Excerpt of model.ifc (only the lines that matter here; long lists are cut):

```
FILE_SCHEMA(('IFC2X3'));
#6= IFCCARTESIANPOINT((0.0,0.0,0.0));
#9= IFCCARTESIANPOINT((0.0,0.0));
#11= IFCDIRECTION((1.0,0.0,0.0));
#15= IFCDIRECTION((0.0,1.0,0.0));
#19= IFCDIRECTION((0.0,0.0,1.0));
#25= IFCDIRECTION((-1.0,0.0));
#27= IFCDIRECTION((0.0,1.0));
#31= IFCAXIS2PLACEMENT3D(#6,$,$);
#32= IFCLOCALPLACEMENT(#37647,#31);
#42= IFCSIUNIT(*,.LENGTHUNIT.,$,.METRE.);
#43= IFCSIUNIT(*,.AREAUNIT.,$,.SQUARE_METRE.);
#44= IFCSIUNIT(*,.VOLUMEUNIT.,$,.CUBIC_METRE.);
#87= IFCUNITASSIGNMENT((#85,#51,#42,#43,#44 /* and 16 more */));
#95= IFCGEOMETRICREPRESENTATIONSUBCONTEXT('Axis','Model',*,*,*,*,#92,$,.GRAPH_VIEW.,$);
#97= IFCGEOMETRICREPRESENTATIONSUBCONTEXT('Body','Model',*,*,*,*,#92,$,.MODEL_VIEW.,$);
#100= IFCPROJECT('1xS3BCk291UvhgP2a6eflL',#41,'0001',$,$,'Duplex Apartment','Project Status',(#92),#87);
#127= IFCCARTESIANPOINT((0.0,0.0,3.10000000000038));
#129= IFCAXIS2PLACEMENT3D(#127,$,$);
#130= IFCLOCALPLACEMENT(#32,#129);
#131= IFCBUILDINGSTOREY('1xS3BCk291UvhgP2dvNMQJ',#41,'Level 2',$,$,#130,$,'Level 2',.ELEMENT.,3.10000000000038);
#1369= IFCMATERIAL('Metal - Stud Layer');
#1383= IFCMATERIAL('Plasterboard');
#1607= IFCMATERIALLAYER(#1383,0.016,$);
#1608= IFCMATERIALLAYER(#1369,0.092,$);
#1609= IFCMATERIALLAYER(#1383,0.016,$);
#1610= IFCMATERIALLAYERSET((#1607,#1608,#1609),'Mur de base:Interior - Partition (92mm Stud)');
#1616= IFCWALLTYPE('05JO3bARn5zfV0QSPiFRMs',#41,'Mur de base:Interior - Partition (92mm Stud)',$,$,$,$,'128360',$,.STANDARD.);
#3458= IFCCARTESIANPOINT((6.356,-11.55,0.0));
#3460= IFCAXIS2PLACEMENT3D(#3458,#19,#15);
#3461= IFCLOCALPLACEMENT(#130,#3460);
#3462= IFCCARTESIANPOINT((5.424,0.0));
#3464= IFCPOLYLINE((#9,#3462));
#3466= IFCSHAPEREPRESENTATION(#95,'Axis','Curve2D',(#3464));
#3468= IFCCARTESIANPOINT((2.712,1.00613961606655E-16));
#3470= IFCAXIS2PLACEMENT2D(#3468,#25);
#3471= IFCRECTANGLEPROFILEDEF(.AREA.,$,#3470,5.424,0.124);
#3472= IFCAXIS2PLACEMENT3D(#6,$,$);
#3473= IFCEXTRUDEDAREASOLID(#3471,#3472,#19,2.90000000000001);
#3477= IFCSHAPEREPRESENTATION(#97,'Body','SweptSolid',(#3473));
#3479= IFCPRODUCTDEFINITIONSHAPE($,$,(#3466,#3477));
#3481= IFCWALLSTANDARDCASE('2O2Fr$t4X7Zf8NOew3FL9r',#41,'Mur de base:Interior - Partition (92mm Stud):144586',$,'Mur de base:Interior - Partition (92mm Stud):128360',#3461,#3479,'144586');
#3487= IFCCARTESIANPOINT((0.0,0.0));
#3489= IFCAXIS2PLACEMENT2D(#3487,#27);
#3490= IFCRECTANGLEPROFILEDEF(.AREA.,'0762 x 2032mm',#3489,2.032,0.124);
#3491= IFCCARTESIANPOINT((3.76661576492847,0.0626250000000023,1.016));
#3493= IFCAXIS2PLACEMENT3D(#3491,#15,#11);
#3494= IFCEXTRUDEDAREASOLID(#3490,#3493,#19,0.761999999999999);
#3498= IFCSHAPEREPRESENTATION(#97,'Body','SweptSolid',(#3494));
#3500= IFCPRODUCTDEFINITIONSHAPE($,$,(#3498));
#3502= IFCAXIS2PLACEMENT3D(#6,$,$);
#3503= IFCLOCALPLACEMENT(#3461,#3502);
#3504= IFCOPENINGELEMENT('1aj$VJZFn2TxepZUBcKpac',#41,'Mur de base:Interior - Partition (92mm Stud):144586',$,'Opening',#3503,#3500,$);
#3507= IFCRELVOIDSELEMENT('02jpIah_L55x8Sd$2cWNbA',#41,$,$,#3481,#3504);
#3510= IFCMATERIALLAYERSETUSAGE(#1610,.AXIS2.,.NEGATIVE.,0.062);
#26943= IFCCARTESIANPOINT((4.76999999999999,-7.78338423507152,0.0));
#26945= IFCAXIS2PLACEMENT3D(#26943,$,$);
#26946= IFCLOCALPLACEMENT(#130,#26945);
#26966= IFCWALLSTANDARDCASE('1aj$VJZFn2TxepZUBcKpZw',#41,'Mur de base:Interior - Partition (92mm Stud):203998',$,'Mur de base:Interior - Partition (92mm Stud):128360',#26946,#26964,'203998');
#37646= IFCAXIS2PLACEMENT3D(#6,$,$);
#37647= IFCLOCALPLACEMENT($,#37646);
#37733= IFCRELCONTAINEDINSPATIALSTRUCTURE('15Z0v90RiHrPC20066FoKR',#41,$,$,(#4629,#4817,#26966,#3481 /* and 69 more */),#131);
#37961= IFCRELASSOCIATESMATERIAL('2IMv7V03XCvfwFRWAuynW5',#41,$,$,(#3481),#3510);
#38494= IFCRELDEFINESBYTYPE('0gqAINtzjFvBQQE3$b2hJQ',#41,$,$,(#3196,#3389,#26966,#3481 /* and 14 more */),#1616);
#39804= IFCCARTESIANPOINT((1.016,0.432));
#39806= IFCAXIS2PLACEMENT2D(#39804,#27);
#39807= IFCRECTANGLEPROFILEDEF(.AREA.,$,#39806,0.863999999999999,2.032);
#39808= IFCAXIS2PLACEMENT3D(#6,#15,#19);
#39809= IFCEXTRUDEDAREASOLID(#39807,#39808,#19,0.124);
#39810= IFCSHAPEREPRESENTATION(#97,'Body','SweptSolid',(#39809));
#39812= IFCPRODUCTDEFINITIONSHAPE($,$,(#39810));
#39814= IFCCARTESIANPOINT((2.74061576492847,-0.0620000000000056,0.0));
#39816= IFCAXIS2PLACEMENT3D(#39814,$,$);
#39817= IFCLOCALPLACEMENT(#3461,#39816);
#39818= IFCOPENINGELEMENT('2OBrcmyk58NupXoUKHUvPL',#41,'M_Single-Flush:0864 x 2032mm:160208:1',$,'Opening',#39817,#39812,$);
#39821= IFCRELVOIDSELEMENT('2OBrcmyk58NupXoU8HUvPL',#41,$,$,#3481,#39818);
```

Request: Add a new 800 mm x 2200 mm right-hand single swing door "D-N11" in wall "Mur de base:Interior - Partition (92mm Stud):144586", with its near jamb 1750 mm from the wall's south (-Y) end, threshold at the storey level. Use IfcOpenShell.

```python
import numpy as np
import ifcopenshell
import ifcopenshell.api.feature
import ifcopenshell.api.geometry
import ifcopenshell.api.root
import ifcopenshell.api.spatial
import ifcopenshell.api.type
import ifcopenshell.geom
import ifcopenshell.util.element
import ifcopenshell.util.placement
import ifcopenshell.util.representation
import ifcopenshell.util.shape
import ifcopenshell.util.unit

model = ifcopenshell.open("model.ifc")
unit_scale = ifcopenshell.util.unit.calculate_unit_scale(model)
settings = ifcopenshell.geom.settings()


def volume(element):
    """Net volume in cubic metres, openings subtracted."""
    shape = ifcopenshell.geom.create_shape(settings, element)
    return ifcopenshell.util.shape.get_volume(shape.geometry)


wall = model.by_guid("2O2Fr$t4X7Zf8NOew3FL9r")
storey = ifcopenshell.util.element.get_container(wall, ifc_class="IfcBuildingStorey")
context = ifcopenshell.util.representation.get_context(model, "Model", "Body", "MODEL_VIEW")
before = volume(wall)

width, height, from_end, sill = 0.8, 2.2, 1.75, 0.0  # metres

# The wall runs along its own X axis, and the end named is its -X end.
wall_shape = ifcopenshell.geom.create_shape(settings, wall)
x, y, z = ifcopenshell.util.shape.get_vertices(wall_shape.geometry).T
start = x.min() + from_end
face, thickness = float(y.min()), float(y.max() - y.min())
wall_matrix = ifcopenshell.util.placement.get_local_placement(wall.ObjectPlacement)
level = ifcopenshell.util.placement.get_local_placement(storey.ObjectPlacement)[2, 3]


def in_wall(x, y):
    """Placement at x, y metres in the wall's axes, at sill height."""
    matrix = wall_matrix.copy()
    matrix[:, 3] = wall_matrix @ np.array([x / unit_scale, y / unit_scale, 0.0, 1.0])
    matrix[2, 3] = level + sill / unit_scale
    return matrix


# Opening: a box that overshoots both wall faces by 50 mm.
opening = ifcopenshell.api.root.create_entity(model, ifc_class="IfcOpeningElement")
box = ifcopenshell.api.geometry.add_wall_representation(
    model, context=context, length=width, height=height, thickness=thickness + 0.1
)
ifcopenshell.api.geometry.assign_representation(model, product=opening, representation=box)
ifcopenshell.api.geometry.edit_object_placement(model, product=opening, matrix=in_wall(start, face - 0.05), is_si=False)
ifcopenshell.api.feature.add_feature(model, feature=opening, element=wall)

door = ifcopenshell.api.root.create_entity(model, ifc_class="IfcDoor", name="D-N11")
door.OverallWidth, door.OverallHeight = width / unit_scale, height / unit_scale
body = ifcopenshell.api.geometry.add_door_representation(
    model,
    context=context,
    overall_width=door.OverallWidth,
    overall_height=door.OverallHeight,
    operation_type="SINGLE_SWING_RIGHT",
    lining_properties={"LiningDepth": thickness / unit_scale, "ThresholdDepth": thickness / unit_scale},
)
ifcopenshell.api.geometry.assign_representation(model, product=door, representation=body)
ifcopenshell.api.spatial.assign_container(model, products=[door], relating_structure=storey)
fills = ifcopenshell.api.feature.add_filling(model, opening=opening, element=door)
fills.OwnerHistory = door.OwnerHistory  # required in IFC2X3

# IFC2X3 keeps the operation on the door style.
style = ifcopenshell.api.root.create_entity(model, ifc_class="IfcDoorStyle", name="D-N11")
style.OperationType, style.ConstructionType = "SINGLE_SWING_RIGHT", "NOTDEFINED"
style.ParameterTakesPrecedence = style.Sizeable = False
ifcopenshell.api.type.assign_type(model, related_objects=[door], relating_type=style)

# The lining spans the wall, so the door starts at the wall face.
ifcopenshell.api.geometry.edit_object_placement(model, product=door, matrix=in_wall(start, face), is_si=False)

after = volume(wall)

print(f"wall volume {before:.3f} -> {after:.3f} m3")

model.write("model_updated.ifc")
```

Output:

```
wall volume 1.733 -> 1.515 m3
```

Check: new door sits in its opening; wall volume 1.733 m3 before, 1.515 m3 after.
